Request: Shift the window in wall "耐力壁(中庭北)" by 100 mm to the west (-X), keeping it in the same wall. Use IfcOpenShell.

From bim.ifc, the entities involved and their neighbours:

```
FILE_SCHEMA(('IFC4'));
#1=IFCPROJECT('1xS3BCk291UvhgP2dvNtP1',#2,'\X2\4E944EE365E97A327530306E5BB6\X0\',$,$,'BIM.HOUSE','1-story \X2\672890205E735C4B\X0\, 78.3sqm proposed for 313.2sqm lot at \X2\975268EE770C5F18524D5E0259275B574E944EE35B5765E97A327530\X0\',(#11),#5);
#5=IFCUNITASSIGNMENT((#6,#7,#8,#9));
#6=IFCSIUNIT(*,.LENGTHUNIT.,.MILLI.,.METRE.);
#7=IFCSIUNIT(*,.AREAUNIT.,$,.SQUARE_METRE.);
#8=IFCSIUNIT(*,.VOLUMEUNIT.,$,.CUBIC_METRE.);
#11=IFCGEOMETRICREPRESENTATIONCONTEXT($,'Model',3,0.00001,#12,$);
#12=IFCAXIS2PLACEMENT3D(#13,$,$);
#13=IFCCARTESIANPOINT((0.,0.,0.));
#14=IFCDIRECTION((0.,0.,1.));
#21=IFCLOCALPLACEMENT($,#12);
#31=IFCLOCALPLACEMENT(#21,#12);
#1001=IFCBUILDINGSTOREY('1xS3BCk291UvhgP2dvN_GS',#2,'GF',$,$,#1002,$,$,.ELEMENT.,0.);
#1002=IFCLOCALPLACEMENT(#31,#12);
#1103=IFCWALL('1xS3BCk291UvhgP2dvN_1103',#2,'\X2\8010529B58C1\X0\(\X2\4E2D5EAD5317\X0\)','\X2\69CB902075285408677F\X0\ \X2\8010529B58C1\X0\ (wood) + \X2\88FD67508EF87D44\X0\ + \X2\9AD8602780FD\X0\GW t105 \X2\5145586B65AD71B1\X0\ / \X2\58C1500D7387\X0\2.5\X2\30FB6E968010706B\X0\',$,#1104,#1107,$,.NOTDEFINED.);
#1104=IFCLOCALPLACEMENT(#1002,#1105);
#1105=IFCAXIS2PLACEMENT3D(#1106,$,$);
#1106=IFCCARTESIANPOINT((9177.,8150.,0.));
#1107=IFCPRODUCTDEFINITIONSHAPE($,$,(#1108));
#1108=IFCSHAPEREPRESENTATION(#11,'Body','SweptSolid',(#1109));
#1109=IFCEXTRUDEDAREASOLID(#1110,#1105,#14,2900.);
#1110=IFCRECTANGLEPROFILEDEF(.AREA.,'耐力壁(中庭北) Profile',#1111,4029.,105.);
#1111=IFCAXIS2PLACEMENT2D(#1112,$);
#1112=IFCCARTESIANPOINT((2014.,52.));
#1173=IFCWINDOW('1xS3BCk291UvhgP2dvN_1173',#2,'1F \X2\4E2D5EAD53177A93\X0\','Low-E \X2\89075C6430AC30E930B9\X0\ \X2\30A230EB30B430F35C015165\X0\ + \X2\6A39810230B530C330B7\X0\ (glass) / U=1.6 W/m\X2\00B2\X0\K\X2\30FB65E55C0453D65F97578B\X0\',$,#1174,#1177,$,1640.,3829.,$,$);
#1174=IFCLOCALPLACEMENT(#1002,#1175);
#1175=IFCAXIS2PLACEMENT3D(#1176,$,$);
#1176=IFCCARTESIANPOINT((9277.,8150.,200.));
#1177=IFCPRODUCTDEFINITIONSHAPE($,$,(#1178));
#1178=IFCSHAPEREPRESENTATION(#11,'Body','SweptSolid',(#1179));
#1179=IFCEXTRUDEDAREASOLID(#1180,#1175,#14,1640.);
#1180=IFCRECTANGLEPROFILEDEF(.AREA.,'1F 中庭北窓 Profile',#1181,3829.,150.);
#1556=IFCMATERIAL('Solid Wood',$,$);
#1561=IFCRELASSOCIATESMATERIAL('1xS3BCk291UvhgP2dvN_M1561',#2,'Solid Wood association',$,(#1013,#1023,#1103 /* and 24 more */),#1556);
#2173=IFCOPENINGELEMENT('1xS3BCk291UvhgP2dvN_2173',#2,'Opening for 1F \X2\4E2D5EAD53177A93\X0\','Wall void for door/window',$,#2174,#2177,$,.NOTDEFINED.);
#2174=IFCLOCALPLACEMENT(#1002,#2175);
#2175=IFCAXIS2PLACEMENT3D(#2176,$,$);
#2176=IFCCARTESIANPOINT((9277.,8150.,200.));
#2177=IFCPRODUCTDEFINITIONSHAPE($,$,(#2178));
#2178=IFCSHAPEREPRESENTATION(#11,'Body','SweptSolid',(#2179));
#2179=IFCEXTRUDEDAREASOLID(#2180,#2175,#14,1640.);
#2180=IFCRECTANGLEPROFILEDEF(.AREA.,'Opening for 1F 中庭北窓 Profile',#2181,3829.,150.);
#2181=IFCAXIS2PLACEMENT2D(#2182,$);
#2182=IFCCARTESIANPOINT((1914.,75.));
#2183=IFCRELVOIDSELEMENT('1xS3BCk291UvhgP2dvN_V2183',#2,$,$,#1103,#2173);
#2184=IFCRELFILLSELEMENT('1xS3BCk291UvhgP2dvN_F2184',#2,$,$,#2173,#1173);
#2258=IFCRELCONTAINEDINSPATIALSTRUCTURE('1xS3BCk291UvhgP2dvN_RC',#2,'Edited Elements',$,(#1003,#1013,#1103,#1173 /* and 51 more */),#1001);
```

```python
import ifcopenshell
import ifcopenshell.api.geometry
import ifcopenshell.util.placement

model = ifcopenshell.open("bim.ifc")

window = model.by_guid("1xS3BCk291UvhgP2dvN_1173")
opening = window.FillsVoids[0].RelatingOpeningElement
wall = opening.VoidsElements[0].RelatingBuildingElement

wall_matrix = ifcopenshell.util.placement.get_local_placement(wall.ObjectPlacement)
shift = wall_matrix[:3, 0] * -100.0
before = ifcopenshell.util.placement.get_local_placement(window.ObjectPlacement)[:3, 3].copy()

# The window is not placed relative to its opening, so move both.
for product in (opening, window):
    matrix = ifcopenshell.util.placement.get_local_placement(product.ObjectPlacement)
    matrix[:3, 3] += shift
    ifcopenshell.api.geometry.edit_object_placement(model, product=product, matrix=matrix, is_si=False)

after = ifcopenshell.util.placement.get_local_placement(window.ObjectPlacement)[:3, 3]
print("window moved by", (after - before).round(3) + 0.0)

model.write("bim_updated.ifc")
```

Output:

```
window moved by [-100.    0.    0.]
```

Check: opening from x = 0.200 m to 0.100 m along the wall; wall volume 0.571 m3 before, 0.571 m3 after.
